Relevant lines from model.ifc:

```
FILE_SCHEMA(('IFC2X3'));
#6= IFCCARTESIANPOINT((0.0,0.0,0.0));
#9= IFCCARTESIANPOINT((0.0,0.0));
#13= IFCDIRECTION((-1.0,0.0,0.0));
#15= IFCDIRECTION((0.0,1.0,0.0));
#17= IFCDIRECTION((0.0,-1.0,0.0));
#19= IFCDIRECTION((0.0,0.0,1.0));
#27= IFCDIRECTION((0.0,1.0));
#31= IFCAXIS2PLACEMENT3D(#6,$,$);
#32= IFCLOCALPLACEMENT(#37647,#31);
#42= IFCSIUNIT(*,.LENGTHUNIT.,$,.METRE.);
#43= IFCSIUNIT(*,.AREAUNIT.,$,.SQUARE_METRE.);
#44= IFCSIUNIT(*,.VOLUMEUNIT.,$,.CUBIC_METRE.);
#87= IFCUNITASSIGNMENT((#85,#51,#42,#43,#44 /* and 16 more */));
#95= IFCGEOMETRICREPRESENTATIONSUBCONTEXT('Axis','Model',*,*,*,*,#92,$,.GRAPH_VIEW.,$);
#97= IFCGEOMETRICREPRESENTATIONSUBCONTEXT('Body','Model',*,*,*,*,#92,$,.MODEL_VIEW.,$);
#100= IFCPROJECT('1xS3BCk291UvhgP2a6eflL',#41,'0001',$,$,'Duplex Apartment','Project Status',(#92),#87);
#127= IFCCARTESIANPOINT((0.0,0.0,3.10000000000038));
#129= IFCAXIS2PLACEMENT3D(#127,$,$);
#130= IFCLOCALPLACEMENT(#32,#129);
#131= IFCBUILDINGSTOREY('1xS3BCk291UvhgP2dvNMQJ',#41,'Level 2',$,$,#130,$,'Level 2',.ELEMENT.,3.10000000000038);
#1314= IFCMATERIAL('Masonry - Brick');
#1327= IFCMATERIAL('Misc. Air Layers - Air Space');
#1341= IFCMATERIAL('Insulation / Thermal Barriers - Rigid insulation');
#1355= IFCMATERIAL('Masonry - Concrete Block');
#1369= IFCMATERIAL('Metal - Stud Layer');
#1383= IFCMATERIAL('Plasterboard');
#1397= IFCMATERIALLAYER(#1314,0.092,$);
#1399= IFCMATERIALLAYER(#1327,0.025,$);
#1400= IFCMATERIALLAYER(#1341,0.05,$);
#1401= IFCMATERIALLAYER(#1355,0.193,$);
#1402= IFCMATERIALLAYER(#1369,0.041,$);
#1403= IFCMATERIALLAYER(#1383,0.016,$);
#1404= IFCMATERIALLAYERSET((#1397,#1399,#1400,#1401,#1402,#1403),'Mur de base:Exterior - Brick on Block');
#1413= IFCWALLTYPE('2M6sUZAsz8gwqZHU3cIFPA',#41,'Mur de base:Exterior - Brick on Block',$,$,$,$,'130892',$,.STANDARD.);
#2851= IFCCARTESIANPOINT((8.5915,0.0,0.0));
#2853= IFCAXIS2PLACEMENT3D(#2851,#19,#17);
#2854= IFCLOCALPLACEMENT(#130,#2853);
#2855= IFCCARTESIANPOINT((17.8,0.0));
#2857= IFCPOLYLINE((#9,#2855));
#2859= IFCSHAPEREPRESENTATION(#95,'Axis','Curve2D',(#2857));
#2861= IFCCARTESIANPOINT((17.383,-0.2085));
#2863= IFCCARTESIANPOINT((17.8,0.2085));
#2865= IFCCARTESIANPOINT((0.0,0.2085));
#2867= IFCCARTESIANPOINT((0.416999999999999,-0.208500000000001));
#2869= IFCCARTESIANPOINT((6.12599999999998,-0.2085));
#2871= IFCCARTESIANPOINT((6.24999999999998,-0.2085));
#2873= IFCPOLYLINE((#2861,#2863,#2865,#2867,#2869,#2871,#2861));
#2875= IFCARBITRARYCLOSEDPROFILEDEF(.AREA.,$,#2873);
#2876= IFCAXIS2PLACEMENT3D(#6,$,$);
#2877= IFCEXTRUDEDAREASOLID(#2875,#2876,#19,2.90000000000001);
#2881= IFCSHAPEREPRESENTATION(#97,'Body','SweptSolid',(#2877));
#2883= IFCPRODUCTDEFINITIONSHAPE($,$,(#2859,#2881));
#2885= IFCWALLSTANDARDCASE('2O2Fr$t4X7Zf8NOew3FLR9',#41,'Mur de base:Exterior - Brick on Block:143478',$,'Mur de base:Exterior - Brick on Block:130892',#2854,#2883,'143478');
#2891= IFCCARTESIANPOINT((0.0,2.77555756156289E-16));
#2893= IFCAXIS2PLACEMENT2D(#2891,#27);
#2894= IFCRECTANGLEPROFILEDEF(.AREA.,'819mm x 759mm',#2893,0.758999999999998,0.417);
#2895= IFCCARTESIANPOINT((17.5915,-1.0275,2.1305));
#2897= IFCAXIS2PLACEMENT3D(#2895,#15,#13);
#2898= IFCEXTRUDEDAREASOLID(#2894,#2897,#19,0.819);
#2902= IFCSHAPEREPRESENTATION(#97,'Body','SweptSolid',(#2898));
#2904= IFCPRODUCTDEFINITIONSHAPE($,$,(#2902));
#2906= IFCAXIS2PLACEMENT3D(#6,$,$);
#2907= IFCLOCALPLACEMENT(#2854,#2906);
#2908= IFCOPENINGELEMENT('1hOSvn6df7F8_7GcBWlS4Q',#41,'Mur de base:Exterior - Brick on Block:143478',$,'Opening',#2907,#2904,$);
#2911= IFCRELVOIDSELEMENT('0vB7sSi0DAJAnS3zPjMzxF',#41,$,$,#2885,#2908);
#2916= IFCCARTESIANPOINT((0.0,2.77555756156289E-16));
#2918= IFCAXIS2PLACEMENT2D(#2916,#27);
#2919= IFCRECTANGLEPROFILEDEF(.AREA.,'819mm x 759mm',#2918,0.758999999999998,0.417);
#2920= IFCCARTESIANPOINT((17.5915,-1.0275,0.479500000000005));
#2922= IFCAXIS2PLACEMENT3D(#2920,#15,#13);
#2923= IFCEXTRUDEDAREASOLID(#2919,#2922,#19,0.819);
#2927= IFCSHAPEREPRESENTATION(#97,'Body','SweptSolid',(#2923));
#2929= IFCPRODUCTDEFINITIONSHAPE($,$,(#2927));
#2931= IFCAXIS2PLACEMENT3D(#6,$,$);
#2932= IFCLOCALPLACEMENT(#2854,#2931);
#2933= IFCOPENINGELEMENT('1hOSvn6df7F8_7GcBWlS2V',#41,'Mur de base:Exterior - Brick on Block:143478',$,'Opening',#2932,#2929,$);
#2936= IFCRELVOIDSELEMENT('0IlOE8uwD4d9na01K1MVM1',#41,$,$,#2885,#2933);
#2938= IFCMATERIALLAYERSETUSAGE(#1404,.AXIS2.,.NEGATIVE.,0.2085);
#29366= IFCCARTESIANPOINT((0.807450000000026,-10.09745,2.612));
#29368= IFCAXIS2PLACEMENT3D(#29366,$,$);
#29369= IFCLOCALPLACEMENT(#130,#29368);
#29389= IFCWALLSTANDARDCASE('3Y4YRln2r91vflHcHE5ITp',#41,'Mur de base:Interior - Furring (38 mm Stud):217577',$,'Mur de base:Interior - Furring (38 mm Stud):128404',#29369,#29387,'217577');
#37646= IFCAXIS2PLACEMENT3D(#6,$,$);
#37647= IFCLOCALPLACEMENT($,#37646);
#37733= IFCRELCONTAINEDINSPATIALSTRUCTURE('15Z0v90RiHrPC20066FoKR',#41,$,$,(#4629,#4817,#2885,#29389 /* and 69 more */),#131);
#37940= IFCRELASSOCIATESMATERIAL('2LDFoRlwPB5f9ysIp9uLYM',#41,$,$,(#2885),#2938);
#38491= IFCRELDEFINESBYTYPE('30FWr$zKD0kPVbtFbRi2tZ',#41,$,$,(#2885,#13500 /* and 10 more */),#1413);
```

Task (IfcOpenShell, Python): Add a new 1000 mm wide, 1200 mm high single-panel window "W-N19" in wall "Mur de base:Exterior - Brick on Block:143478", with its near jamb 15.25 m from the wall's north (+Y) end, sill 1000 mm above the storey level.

```python
import numpy as np
import ifcopenshell
import ifcopenshell.api.feature
import ifcopenshell.api.geometry
import ifcopenshell.api.root
import ifcopenshell.api.spatial
import ifcopenshell.api.type
import ifcopenshell.geom
import ifcopenshell.util.element
import ifcopenshell.util.placement
import ifcopenshell.util.representation
import ifcopenshell.util.shape
import ifcopenshell.util.unit

model = ifcopenshell.open("model.ifc")
unit_scale = ifcopenshell.util.unit.calculate_unit_scale(model)
settings = ifcopenshell.geom.settings()


def volume(element):
    """Net volume in cubic metres, openings subtracted."""
    shape = ifcopenshell.geom.create_shape(settings, element)
    return ifcopenshell.util.shape.get_volume(shape.geometry)


wall = model.by_guid("2O2Fr$t4X7Zf8NOew3FLR9")
storey = ifcopenshell.util.element.get_container(wall, ifc_class="IfcBuildingStorey")
context = ifcopenshell.util.representation.get_context(model, "Model", "Body", "MODEL_VIEW")
before = volume(wall)

width, height, from_end, sill = 1, 1.2, 15.25, 1  # metres

# The wall runs along its own X axis, and the end named is its -X end.
wall_shape = ifcopenshell.geom.create_shape(settings, wall)
x, y, z = ifcopenshell.util.shape.get_vertices(wall_shape.geometry).T
start = x.min() + from_end
face, thickness = float(y.min()), float(y.max() - y.min())
wall_matrix = ifcopenshell.util.placement.get_local_placement(wall.ObjectPlacement)
level = ifcopenshell.util.placement.get_local_placement(storey.ObjectPlacement)[2, 3]


def in_wall(x, y):
    """Placement at x, y metres in the wall's axes, at sill height."""
    matrix = wall_matrix.copy()
    matrix[:, 3] = wall_matrix @ np.array([x / unit_scale, y / unit_scale, 0.0, 1.0])
    matrix[2, 3] = level + sill / unit_scale
    return matrix


# Opening: a box that overshoots both wall faces by 50 mm.
opening = ifcopenshell.api.root.create_entity(model, ifc_class="IfcOpeningElement")
box = ifcopenshell.api.geometry.add_wall_representation(
    model, context=context, length=width, height=height, thickness=thickness + 0.1
)
ifcopenshell.api.geometry.assign_representation(model, product=opening, representation=box)
ifcopenshell.api.geometry.edit_object_placement(model, product=opening, matrix=in_wall(start, face - 0.05), is_si=False)
ifcopenshell.api.feature.add_feature(model, feature=opening, element=wall)

window = ifcopenshell.api.root.create_entity(model, ifc_class="IfcWindow", name="W-N19")
window.OverallWidth, window.OverallHeight = width / unit_scale, height / unit_scale
body = ifcopenshell.api.geometry.add_window_representation(
    model,
    context=context,
    overall_width=window.OverallWidth,
    overall_height=window.OverallHeight,
    partition_type="SINGLE_PANEL",
)
ifcopenshell.api.geometry.assign_representation(model, product=window, representation=body)
ifcopenshell.api.spatial.assign_container(model, products=[window], relating_structure=storey)
fills = ifcopenshell.api.feature.add_filling(model, opening=opening, element=window)
fills.OwnerHistory = window.OwnerHistory  # required in IFC2X3

# IFC2X3 keeps the operation on the window style.
style = ifcopenshell.api.root.create_entity(model, ifc_class="IfcWindowStyle", name="W-N19")
style.OperationType, style.ConstructionType = "SINGLE_PANEL", "NOTDEFINED"
style.ParameterTakesPrecedence = style.Sizeable = False
ifcopenshell.api.type.assign_type(model, related_objects=[window], relating_type=style)

# Centre the window in the wall's thickness.
ifcopenshell.api.geometry.edit_object_placement(model, product=window, matrix=in_wall(start, face), is_si=False)
window_shape = ifcopenshell.geom.create_shape(settings, window)
depth = ifcopenshell.util.shape.get_vertices(window_shape.geometry)[:, 1]
offset = face + thickness / 2 - (depth.min() + depth.max()) / 2
ifcopenshell.api.geometry.edit_object_placement(model, product=window, matrix=in_wall(start, offset), is_si=False)

after = volume(wall)

print(f"wall volume {before:.3f} -> {after:.3f} m3")

model.write("model_rev.ifc")
```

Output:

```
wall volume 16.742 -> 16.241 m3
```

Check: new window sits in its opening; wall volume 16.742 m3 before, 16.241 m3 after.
